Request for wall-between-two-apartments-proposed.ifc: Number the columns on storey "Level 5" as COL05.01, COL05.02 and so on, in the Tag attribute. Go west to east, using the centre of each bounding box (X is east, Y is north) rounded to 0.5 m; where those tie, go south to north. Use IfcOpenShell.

First a look at what the model holds.

```python
import ifcopenshell
import ifcopenshell.util.element
import ifcopenshell.util.placement

model = ifcopenshell.open("wall-between-two-apartments-proposed.ifc")
print(model.schema)
storey = next(s for s in model.by_type("IfcBuildingStorey") if s.Name == "Level 5")
columns = [e for e in ifcopenshell.util.element.get_decomposition(storey) if e.is_a("IfcColumn")]
for e in sorted(columns, key=lambda e: e.id()):
    origin = ifcopenshell.util.placement.get_local_placement(e.ObjectPlacement)[:3, 3]
    print(e.id(), e.Tag, e.Name, origin.round(2) + 0.0, sep=" | ")
```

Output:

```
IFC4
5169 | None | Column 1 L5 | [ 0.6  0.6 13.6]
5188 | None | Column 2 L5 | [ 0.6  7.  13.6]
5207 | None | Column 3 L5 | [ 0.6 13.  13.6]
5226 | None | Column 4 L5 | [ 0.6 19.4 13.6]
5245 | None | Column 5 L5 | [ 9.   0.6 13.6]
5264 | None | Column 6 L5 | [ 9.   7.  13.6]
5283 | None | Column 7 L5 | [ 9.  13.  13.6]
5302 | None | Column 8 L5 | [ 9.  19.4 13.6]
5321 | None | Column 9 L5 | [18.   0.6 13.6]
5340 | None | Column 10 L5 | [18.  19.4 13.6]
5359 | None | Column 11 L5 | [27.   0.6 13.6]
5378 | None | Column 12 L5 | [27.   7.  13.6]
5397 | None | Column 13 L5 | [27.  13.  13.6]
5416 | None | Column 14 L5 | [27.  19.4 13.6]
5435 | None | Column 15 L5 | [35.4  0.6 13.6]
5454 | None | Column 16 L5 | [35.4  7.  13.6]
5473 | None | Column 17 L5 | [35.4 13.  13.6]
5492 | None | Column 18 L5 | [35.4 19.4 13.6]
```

```python
import ifcopenshell
import ifcopenshell.geom
import ifcopenshell.util.element
import ifcopenshell.util.shape

model = ifcopenshell.open("wall-between-two-apartments-proposed.ifc")
settings = ifcopenshell.geom.settings()
settings.set("use-world-coords", True)


def centre(element):
    shape = ifcopenshell.geom.create_shape(settings, element)
    return ifcopenshell.util.shape.get_bbox_centroid(shape.geometry)


storey = next(s for s in model.by_type("IfcBuildingStorey") if s.Name == "Level 5")
columns = [e for e in ifcopenshell.util.element.get_decomposition(storey) if e.is_a("IfcColumn")]

# Insertion points can sit at a corner or the storey origin, so sort by the geometry (in metres).
centres = {e: centre(e) for e in columns}
columns.sort(key=lambda e: (round(centres[e][0] / 0.5), centres[e][1]))

for i, e in enumerate(columns, start=1):
    number = f"COL05.{i:02d}"
    e.Tag = number
    print(e.id(), number)

model.write("wall-between-two-apartments-proposed_updated.ifc")
```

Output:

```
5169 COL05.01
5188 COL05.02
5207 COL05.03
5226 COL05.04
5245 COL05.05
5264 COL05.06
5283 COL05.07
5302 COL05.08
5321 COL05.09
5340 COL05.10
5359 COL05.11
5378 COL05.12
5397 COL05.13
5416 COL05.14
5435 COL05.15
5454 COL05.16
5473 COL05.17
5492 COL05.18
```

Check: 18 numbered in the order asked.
